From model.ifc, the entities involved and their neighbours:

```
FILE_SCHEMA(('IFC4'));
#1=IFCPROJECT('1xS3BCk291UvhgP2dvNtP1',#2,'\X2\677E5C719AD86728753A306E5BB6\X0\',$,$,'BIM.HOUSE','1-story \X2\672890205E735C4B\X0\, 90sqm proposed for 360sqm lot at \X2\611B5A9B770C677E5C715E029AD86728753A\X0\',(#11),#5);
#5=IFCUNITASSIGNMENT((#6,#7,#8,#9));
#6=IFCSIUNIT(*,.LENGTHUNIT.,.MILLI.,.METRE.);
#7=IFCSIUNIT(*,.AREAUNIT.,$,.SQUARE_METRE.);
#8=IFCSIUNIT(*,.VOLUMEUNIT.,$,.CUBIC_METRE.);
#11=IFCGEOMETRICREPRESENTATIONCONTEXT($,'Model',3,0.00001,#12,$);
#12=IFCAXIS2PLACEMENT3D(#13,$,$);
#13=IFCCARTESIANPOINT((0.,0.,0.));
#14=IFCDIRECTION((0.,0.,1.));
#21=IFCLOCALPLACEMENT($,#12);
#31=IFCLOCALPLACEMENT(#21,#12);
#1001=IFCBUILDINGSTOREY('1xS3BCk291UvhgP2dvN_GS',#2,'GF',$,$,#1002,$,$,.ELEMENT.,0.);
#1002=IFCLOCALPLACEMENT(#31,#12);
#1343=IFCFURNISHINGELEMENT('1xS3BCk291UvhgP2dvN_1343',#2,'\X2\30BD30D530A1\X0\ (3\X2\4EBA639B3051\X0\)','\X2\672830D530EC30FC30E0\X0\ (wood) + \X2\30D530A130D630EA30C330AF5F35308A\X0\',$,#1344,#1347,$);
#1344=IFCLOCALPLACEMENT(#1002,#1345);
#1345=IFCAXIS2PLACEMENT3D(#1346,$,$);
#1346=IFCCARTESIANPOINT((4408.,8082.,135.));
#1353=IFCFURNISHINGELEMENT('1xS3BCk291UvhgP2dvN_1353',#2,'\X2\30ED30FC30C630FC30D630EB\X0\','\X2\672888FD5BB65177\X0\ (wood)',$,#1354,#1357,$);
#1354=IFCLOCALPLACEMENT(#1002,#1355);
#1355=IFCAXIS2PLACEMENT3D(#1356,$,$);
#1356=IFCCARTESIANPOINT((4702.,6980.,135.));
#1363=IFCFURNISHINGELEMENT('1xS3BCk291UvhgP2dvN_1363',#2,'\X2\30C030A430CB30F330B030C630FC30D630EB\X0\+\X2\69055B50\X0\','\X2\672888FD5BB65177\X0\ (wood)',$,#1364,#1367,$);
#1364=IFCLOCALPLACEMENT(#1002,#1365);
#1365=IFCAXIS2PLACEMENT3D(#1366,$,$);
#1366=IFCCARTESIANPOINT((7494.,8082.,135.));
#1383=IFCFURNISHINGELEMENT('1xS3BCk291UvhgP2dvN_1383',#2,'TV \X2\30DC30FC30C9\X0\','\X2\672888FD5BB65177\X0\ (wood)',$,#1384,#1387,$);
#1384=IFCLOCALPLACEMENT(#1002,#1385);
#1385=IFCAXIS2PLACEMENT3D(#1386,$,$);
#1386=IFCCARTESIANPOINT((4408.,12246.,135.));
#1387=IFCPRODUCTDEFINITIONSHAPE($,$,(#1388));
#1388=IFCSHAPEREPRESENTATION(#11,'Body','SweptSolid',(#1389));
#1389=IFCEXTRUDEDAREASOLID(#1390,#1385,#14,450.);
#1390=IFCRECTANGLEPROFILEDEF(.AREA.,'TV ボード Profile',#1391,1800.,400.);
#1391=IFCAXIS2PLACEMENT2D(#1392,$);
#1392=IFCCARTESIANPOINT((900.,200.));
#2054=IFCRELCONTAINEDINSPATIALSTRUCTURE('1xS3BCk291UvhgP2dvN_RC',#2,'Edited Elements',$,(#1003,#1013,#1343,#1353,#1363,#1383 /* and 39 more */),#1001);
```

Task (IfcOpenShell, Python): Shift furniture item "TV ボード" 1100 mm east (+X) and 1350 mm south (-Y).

```python
import ifcopenshell
import ifcopenshell.api.geometry
import ifcopenshell.util.placement
import ifcopenshell.util.unit

model = ifcopenshell.open("model.ifc")
unit_scale = ifcopenshell.util.unit.calculate_unit_scale(model)

item = model.by_id(1383)
matrix = ifcopenshell.util.placement.get_local_placement(item.ObjectPlacement)
matrix[0, 3] += 1.1 / unit_scale
matrix[1, 3] -= 1.35 / unit_scale
ifcopenshell.api.geometry.edit_object_placement(model, product=item, matrix=matrix, is_si=False)

print(ifcopenshell.util.placement.get_local_placement(item.ObjectPlacement).round(3) + 0.0)

model.write("model_edited.ifc")
```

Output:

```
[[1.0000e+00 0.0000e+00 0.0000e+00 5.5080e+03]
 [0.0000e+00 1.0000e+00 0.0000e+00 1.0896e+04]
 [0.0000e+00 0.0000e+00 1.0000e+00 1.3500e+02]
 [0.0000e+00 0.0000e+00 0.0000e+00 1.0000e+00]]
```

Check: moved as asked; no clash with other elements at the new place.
